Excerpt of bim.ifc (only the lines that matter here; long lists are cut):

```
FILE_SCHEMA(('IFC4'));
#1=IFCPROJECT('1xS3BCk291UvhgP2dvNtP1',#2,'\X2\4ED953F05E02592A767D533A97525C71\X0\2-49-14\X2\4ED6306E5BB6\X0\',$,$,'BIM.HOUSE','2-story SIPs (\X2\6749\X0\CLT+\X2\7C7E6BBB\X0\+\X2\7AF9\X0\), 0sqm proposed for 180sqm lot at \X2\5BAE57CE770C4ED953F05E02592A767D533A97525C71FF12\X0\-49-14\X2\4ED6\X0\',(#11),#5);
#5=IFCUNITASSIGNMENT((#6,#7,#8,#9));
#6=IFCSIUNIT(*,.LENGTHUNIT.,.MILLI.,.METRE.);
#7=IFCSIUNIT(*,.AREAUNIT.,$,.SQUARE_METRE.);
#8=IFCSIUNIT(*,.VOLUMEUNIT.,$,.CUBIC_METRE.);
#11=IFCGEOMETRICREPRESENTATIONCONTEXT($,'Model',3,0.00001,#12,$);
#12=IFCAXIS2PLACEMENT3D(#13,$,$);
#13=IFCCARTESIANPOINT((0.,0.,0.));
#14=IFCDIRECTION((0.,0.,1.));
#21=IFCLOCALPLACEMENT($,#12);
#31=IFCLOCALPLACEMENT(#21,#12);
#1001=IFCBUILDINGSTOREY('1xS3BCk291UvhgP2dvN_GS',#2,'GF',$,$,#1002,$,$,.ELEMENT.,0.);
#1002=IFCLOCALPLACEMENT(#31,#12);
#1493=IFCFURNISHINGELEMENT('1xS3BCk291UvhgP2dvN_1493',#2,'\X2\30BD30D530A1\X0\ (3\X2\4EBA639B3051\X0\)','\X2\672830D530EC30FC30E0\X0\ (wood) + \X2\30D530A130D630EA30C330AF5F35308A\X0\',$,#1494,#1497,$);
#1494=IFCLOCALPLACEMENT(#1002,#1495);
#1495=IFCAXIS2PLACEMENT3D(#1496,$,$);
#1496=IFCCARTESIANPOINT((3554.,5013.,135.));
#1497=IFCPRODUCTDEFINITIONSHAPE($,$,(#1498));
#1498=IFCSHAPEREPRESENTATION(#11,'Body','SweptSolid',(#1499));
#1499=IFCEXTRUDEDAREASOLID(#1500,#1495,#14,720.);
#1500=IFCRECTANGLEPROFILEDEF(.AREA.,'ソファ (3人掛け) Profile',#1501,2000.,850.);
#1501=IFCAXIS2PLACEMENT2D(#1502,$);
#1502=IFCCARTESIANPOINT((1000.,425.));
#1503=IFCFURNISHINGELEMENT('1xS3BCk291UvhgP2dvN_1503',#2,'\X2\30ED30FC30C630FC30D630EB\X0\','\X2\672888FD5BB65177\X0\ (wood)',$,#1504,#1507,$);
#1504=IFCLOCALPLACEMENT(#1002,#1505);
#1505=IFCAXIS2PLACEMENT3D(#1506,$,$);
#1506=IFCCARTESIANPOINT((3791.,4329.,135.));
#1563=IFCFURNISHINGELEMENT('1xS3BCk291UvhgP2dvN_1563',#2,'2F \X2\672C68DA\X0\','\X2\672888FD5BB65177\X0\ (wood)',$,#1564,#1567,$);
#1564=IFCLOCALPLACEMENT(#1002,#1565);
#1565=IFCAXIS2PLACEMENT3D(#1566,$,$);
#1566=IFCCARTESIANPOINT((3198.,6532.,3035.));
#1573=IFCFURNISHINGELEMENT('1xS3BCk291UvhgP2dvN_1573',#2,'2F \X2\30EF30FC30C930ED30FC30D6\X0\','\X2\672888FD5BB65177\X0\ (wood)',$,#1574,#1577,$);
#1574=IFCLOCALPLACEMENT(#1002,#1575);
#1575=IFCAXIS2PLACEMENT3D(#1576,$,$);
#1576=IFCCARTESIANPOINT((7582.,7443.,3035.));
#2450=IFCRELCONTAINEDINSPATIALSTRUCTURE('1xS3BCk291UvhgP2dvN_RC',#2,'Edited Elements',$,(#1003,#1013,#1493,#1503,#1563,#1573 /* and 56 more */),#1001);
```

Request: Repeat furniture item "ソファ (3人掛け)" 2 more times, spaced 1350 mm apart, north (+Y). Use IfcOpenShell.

```python
import numpy as np
import ifcopenshell
import ifcopenshell.api.geometry
import ifcopenshell.api.root
import ifcopenshell.util.element
import ifcopenshell.util.placement
import ifcopenshell.util.unit

model = ifcopenshell.open("bim.ifc")
unit_scale = ifcopenshell.util.unit.calculate_unit_scale(model)


def reuse_history(source, copy):
    """copy_class also copies each property set's owner history, people and application; keep the originals."""
    for rel in copy.IsDefinedBy:
        if rel.is_a("IfcRelDefinesByProperties") and (history := rel.RelatingPropertyDefinition.OwnerHistory):
            rel.RelatingPropertyDefinition.OwnerHistory = source.OwnerHistory
            ifcopenshell.util.element.remove_deep2(model, history)


source = model.by_id(1493)
base = ifcopenshell.util.placement.get_local_placement(source.ObjectPlacement)
step = np.array([0.0, 1.0, 0.0]) * 1.35 / unit_scale

for i in range(1, 3):
    copy = ifcopenshell.api.root.copy_class(model, product=source)
    copy.Representation = ifcopenshell.util.element.copy_deep(
        model, source.Representation, exclude=["IfcGeometricRepresentationContext", "IfcRepresentationMap"]
    )
    reuse_history(source, copy)
    matrix = base.copy()
    matrix[:3, 3] += i * step
    print("added at", matrix[:3, 3].round(3) + 0.0)
    ifcopenshell.api.geometry.edit_object_placement(model, product=copy, matrix=matrix, is_si=False)

model.write("bim_v2.ifc")
```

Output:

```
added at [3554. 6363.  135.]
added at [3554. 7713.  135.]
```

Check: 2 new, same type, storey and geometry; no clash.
